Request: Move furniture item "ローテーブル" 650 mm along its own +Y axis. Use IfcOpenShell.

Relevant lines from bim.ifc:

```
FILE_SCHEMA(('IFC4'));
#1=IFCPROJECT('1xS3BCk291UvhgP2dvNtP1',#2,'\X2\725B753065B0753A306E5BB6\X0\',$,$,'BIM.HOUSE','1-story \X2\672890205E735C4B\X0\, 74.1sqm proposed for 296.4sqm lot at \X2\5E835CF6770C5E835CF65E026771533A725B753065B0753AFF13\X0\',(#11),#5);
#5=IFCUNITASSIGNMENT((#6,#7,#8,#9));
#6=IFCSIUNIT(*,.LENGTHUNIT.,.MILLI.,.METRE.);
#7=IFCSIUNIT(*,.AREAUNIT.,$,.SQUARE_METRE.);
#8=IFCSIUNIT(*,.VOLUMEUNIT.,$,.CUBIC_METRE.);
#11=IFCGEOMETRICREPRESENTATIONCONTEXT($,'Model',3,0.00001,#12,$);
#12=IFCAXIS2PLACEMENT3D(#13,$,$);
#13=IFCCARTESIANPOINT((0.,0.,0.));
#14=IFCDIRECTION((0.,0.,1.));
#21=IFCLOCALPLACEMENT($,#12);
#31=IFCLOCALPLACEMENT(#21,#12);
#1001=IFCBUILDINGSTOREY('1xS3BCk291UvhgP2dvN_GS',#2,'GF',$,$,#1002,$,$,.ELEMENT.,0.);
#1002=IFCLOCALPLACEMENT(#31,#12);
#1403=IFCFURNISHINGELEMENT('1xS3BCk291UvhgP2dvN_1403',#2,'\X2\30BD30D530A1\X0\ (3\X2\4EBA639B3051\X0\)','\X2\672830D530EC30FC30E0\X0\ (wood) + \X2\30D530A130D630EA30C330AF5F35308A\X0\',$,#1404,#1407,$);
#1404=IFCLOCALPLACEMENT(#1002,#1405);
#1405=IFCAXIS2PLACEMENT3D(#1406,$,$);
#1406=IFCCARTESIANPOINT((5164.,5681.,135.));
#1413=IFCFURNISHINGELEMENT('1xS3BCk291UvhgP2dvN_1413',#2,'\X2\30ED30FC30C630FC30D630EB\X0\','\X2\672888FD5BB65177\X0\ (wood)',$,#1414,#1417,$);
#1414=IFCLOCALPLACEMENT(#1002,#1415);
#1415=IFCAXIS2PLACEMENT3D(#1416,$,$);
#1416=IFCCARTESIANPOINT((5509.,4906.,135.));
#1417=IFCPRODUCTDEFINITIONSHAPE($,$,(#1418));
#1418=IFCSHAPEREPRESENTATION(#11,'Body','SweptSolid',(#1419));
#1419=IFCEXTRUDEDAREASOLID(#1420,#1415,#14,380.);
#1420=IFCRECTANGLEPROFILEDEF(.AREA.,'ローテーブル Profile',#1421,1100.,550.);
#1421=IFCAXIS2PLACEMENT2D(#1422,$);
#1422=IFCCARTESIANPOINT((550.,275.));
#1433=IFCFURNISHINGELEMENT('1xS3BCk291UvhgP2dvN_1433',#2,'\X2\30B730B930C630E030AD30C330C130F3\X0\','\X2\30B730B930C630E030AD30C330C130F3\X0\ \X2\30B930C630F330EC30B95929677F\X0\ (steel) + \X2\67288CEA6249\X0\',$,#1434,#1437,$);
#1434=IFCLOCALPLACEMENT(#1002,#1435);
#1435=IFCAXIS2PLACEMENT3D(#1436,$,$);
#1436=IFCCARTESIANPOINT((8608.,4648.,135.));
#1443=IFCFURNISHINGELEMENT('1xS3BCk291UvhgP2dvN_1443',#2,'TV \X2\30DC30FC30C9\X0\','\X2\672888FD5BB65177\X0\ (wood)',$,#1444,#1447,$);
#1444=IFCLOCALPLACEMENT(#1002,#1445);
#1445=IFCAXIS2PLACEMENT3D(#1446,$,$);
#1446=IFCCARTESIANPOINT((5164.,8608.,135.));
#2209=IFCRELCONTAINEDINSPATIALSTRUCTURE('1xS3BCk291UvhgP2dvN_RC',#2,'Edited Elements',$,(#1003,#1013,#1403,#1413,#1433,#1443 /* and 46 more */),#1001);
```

```python
import ifcopenshell
import ifcopenshell.api.geometry
import ifcopenshell.util.placement

model = ifcopenshell.open("bim.ifc")

item = model.by_id(1413)
matrix = ifcopenshell.util.placement.get_local_placement(item.ObjectPlacement)
matrix[:3, 3] += matrix[:3, 1] * 650.0
ifcopenshell.api.geometry.edit_object_placement(model, product=item, matrix=matrix, is_si=False)

print(ifcopenshell.util.placement.get_local_placement(item.ObjectPlacement).round(3) + 0.0)

model.write("bim_v2.ifc")
```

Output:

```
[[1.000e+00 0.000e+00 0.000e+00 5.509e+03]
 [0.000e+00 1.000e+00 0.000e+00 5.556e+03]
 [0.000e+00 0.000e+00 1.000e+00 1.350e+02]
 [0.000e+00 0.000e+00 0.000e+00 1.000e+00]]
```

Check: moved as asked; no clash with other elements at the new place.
